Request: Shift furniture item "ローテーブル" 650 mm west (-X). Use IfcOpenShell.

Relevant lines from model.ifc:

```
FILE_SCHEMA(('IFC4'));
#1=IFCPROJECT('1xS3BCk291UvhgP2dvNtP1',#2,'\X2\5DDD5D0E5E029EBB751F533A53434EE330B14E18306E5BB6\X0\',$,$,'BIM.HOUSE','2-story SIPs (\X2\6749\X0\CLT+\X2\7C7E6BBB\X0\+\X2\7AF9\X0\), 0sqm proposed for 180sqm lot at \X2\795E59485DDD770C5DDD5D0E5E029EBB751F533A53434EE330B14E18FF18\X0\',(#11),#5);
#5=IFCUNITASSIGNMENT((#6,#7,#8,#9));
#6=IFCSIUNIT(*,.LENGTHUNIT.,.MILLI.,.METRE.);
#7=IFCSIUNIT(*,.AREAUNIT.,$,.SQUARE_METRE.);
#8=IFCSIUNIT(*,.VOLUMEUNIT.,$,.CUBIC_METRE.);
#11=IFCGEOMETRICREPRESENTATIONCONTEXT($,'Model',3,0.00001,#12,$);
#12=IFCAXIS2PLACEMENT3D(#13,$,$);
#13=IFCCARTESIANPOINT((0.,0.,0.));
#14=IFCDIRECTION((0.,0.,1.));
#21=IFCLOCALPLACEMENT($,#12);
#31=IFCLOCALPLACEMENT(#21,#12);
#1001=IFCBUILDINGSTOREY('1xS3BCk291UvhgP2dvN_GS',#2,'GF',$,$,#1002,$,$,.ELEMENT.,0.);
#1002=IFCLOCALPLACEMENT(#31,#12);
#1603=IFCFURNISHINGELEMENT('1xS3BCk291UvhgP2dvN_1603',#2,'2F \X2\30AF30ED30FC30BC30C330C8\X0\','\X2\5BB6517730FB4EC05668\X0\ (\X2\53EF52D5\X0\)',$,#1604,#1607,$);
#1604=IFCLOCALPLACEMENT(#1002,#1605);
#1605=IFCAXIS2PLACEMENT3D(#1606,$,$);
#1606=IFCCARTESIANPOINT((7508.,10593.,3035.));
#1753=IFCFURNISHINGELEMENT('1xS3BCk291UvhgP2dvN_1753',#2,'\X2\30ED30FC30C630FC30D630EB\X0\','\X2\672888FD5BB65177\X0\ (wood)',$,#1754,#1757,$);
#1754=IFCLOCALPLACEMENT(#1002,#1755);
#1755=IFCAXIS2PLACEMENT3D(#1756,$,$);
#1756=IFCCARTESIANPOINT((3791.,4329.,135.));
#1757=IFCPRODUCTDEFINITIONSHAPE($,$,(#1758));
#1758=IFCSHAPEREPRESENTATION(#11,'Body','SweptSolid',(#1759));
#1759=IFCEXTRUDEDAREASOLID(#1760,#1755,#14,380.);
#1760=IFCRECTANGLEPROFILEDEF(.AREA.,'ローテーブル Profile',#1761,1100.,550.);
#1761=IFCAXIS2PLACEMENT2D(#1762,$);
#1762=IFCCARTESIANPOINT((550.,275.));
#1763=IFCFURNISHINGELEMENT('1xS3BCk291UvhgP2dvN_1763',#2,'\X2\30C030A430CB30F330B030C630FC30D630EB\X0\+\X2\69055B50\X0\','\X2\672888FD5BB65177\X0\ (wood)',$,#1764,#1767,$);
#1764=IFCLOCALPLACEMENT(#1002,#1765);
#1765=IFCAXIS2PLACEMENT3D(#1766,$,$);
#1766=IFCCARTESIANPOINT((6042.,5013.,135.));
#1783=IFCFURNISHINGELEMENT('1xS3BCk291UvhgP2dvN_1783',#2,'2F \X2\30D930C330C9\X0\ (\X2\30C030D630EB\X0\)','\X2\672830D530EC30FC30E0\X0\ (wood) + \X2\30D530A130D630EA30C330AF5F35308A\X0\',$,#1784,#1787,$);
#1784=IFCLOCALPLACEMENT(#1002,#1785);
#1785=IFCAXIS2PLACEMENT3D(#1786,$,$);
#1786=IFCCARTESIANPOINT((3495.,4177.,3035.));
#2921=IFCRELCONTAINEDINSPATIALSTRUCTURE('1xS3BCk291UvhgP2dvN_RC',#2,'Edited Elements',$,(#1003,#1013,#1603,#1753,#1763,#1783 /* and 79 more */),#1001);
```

```python
import ifcopenshell
import ifcopenshell.api.geometry
import ifcopenshell.util.placement
import ifcopenshell.util.unit

model = ifcopenshell.open("model.ifc")
unit_scale = ifcopenshell.util.unit.calculate_unit_scale(model)

item = model.by_guid("1xS3BCk291UvhgP2dvN_1753")
matrix = ifcopenshell.util.placement.get_local_placement(item.ObjectPlacement)
matrix[0, 3] -= 0.65 / unit_scale
ifcopenshell.api.geometry.edit_object_placement(model, product=item, matrix=matrix, is_si=False)

print(ifcopenshell.util.placement.get_local_placement(item.ObjectPlacement).round(3) + 0.0)

model.write("model_updated.ifc")
```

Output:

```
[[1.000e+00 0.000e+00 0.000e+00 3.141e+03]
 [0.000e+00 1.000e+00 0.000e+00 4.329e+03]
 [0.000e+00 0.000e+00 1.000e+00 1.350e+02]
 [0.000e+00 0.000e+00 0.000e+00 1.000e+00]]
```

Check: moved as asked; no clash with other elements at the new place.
